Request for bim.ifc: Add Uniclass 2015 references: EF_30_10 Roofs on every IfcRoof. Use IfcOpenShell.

First a look at what the model holds.

```python
import ifcopenshell

model = ifcopenshell.open("bim.ifc")
print(model.schema)
print("classifications:", [c.Name for c in model.by_type("IfcClassification")])
for ifc_class in ("IfcDoor", "IfcRoof", "IfcStair", "IfcWall", "IfcWindow"):
    print(ifc_class, len(model.by_type(ifc_class)))
```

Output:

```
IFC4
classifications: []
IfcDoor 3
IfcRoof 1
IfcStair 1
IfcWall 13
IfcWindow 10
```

```python
import ifcopenshell
import ifcopenshell.api.classification

model = ifcopenshell.open("bim.ifc")

system = ifcopenshell.api.classification.add_classification(model, classification="Uniclass 2015")

codes = {
    "IfcRoof": ("EF_30_10", "Roofs"),
}
for ifc_class, (code, name) in codes.items():
    products = model.by_type(ifc_class)
    ifcopenshell.api.classification.add_reference(
        model, products=products, classification=system, identification=code, name=name
    )
    print(code, len(products))

model.write("bim_v2.ifc")
```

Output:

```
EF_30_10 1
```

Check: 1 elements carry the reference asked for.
